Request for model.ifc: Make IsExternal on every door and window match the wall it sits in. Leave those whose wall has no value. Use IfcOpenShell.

First a look at what the model holds.

```python
import ifcopenshell
import ifcopenshell.util.element

model = ifcopenshell.open("model.ifc")
print(model.schema)
seen = {}
for e in model.by_type("IfcDoor") + model.by_type("IfcWindow"):
    if not e.FillsVoids:
        continue
    host = e.FillsVoids[0].RelatingOpeningElement.VoidsElements[0].RelatingBuildingElement
    own = ifcopenshell.util.element.get_pset(e, f"Pset_{e.is_a()[3:].removesuffix('StandardCase')}Common", "IsExternal")
    wall = ifcopenshell.util.element.get_pset(host, "Pset_WallCommon", "IsExternal")
    seen[e.is_a(), own, wall] = seen.get((e.is_a(), own, wall), 0) + 1
for (cls, own, wall), count in sorted(seen.items(), key=str):
    print(count, cls, "IsExternal:", own, "| host wall:", wall)
```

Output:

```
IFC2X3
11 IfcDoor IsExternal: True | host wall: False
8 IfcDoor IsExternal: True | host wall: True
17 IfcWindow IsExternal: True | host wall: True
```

```python
import ifcopenshell
import ifcopenshell.api.pset
import ifcopenshell.util.element

model = ifcopenshell.open("model.ifc")

count = 0
for ifc_class, pset_name in (("IfcDoor", "Pset_DoorCommon"), ("IfcWindow", "Pset_WindowCommon")):
    for e in model.by_type(ifc_class):
        if not e.FillsVoids:
            continue
        host = e.FillsVoids[0].RelatingOpeningElement.VoidsElements[0].RelatingBuildingElement
        external = ifcopenshell.util.element.get_pset(host, "Pset_WallCommon", "IsExternal")
        if external is None or ifcopenshell.util.element.get_pset(e, pset_name, "IsExternal") == external:
            continue
        pset = ifcopenshell.api.pset.add_pset(model, product=e, name=pset_name)
        ifcopenshell.api.pset.edit_pset(model, pset=pset, properties={"IsExternal": external})
        count += 1

print(count, "updated")

model.write("model_v2.ifc")
```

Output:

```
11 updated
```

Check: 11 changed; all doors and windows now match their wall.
